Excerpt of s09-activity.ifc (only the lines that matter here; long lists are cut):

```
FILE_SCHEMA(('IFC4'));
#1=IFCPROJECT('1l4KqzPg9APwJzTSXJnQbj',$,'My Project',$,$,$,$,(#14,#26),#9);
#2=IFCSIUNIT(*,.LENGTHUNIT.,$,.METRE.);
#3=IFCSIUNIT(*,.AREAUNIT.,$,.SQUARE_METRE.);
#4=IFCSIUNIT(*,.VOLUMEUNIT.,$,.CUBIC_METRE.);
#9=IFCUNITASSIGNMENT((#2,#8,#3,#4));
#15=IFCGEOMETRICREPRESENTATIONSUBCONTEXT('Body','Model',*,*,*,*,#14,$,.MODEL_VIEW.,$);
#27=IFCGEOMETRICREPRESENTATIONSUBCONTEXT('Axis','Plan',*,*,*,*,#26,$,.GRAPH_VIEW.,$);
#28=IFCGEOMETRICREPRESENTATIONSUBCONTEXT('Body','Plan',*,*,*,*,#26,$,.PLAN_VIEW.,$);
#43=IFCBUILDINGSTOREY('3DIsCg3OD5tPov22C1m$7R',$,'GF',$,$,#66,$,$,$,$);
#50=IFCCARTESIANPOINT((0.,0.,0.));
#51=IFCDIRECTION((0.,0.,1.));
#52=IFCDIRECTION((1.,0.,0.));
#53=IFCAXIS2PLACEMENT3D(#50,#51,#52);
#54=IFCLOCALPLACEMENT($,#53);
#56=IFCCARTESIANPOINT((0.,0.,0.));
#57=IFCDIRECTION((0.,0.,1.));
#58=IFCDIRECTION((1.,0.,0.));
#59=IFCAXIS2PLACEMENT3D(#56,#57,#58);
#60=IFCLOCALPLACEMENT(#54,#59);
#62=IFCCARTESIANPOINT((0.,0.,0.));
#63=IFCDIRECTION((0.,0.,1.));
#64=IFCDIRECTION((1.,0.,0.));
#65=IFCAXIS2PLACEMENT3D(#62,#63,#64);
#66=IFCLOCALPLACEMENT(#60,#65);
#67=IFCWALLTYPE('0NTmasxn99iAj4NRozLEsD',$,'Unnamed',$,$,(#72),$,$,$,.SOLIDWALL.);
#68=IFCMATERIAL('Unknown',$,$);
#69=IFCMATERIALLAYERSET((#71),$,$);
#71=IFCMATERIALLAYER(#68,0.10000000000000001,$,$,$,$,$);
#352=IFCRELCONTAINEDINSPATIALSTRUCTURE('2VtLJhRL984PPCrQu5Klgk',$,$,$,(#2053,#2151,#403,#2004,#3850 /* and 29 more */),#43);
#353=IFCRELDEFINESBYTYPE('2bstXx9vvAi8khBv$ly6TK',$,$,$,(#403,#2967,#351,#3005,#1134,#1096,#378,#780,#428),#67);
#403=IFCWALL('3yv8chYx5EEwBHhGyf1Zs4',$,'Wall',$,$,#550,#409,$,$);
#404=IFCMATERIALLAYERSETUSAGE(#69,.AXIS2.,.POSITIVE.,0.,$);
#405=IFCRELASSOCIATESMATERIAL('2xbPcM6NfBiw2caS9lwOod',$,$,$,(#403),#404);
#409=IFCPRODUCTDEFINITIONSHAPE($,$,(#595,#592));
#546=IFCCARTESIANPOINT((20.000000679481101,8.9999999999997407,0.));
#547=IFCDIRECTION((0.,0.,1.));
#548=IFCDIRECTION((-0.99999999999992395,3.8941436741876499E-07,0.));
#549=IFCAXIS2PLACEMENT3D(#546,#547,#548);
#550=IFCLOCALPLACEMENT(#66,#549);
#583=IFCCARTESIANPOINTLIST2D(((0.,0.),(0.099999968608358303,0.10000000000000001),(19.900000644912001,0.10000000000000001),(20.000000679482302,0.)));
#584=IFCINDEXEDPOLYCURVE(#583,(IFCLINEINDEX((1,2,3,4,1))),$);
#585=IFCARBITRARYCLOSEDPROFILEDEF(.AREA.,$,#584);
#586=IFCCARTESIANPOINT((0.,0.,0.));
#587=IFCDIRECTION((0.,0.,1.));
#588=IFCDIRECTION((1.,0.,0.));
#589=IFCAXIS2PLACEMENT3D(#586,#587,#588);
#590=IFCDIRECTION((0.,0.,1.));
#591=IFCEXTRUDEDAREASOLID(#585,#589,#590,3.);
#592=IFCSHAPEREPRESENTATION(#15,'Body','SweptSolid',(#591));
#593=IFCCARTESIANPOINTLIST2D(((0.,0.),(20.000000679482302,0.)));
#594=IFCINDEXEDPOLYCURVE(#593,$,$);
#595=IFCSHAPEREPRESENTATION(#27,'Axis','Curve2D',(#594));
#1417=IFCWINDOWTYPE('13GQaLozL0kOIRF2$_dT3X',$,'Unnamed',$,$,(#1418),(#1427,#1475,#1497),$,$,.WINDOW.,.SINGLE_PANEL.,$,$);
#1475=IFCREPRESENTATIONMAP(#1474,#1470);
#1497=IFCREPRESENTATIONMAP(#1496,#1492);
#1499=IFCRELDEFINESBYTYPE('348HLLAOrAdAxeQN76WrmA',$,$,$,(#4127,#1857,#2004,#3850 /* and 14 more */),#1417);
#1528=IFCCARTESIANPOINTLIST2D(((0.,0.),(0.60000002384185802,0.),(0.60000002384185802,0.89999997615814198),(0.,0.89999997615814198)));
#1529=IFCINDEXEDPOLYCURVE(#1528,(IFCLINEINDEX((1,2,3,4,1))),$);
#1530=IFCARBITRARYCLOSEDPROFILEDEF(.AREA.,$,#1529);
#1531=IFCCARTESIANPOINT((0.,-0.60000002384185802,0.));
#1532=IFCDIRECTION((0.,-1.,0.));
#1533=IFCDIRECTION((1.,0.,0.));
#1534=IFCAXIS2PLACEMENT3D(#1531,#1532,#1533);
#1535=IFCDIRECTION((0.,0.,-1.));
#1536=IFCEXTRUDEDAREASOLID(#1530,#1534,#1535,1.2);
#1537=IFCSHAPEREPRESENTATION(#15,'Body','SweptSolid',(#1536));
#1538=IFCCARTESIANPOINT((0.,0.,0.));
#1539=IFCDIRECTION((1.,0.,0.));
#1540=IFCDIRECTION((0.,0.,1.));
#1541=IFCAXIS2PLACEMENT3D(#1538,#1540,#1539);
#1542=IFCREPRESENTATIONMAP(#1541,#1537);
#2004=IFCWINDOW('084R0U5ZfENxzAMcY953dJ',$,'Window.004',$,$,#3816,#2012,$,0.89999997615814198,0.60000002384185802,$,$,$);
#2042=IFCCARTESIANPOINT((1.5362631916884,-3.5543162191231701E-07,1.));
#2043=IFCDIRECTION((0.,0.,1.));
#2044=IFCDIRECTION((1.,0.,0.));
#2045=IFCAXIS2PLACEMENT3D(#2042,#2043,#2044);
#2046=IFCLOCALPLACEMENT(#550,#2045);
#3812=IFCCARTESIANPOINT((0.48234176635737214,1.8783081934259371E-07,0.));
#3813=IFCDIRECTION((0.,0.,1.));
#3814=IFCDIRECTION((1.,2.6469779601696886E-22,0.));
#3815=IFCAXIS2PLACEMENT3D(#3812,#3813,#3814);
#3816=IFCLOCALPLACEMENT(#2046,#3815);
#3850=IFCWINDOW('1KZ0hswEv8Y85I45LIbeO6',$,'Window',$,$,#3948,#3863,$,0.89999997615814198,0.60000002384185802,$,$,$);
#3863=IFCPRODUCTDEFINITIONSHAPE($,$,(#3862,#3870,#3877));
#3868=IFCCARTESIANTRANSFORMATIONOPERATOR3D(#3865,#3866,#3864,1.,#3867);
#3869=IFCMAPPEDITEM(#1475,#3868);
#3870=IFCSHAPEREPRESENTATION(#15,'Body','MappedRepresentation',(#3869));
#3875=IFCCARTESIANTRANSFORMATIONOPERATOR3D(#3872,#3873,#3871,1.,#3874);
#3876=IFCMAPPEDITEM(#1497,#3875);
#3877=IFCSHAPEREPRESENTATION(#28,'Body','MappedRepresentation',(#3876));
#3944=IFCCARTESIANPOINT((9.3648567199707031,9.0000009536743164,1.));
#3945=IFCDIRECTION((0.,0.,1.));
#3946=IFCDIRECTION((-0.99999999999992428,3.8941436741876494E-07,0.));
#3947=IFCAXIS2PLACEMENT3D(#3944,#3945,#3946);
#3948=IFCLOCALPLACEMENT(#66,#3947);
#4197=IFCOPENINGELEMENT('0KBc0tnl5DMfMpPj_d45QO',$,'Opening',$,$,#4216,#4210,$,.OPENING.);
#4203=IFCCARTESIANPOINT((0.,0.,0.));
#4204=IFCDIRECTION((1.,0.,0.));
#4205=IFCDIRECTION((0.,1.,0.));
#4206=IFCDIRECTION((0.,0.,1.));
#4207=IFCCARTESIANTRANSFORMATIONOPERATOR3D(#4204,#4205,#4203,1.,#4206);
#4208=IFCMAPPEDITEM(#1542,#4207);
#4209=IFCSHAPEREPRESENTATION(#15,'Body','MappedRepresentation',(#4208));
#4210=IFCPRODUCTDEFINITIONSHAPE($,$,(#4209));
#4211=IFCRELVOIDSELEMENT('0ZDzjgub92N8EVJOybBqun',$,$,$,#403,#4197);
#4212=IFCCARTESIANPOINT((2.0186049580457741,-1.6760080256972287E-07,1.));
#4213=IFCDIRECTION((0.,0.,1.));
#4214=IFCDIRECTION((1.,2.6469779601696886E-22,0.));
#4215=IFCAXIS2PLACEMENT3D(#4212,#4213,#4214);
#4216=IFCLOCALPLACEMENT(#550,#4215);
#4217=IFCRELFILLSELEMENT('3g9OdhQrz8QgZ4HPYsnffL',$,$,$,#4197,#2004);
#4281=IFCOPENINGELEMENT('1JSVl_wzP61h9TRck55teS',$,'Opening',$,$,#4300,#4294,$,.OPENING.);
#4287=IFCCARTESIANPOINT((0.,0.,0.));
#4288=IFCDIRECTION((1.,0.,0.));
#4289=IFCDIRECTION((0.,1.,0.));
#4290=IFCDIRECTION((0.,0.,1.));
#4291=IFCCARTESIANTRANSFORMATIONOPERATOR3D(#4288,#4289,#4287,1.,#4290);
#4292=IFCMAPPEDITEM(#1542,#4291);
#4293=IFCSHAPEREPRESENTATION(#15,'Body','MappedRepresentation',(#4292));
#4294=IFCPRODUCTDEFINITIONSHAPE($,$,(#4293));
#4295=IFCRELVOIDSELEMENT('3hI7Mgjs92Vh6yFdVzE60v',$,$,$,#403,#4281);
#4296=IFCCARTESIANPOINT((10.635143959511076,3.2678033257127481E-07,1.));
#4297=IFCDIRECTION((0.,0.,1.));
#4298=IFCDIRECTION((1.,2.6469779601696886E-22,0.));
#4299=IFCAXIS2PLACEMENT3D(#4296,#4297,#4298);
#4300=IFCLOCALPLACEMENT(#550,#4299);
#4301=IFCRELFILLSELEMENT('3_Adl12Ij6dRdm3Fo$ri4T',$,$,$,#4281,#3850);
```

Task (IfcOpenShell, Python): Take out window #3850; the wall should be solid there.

```python
import ifcopenshell
import ifcopenshell.api.feature
import ifcopenshell.api.root
import ifcopenshell.geom
import ifcopenshell.util.shape

model = ifcopenshell.open("s09-activity.ifc")
settings = ifcopenshell.geom.settings()


def volume(element):
    """Net volume in cubic metres, openings subtracted."""
    shape = ifcopenshell.geom.create_shape(settings, element)
    return ifcopenshell.util.shape.get_volume(shape.geometry)


window = model.by_id(3850)
opening = window.FillsVoids[0].RelatingOpeningElement
wall = opening.VoidsElements[0].RelatingBuildingElement
before = volume(wall)

ifcopenshell.api.root.remove_product(model, product=window)
ifcopenshell.api.feature.remove_feature(model, feature=opening)

after = volume(wall)

print(f"wall volume {before:.3f} -> {after:.3f} m3")

model.write("s09-activity_edited.ifc")
```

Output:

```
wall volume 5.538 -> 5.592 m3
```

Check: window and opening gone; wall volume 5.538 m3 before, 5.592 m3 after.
